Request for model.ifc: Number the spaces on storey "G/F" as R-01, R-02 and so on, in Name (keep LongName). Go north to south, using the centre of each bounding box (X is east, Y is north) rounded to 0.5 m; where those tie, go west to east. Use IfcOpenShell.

First a look at what the model holds.

```python
import ifcopenshell
import ifcopenshell.util.element
import ifcopenshell.util.placement

model = ifcopenshell.open("model.ifc")
print(model.schema)
storey = next(s for s in model.by_type("IfcBuildingStorey") if s.Name == "G/F")
spaces = [e for e in ifcopenshell.util.element.get_decomposition(storey) if e.is_a("IfcSpace")]
for e in sorted(spaces, key=lambda e: e.id()):
    origin = ifcopenshell.util.placement.get_local_placement(e.ObjectPlacement)[:3, 3]
    print(e.id(), e.Name, e.LongName, origin.round(2) + 0.0, sep=" | ")
```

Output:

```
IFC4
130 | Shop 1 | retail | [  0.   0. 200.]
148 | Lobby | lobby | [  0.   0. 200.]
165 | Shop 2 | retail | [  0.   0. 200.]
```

```python
import ifcopenshell
import ifcopenshell.geom
import ifcopenshell.util.element
import ifcopenshell.util.shape

model = ifcopenshell.open("model.ifc")
settings = ifcopenshell.geom.settings()
settings.set("use-world-coords", True)


def centre(element):
    shape = ifcopenshell.geom.create_shape(settings, element)
    return ifcopenshell.util.shape.get_bbox_centroid(shape.geometry)


storey = next(s for s in model.by_type("IfcBuildingStorey") if s.Name == "G/F")
spaces = [e for e in ifcopenshell.util.element.get_decomposition(storey) if e.is_a("IfcSpace")]

# Insertion points can sit at a corner or the storey origin, so sort by the geometry (in metres).
centres = {e: centre(e) for e in spaces}
spaces.sort(key=lambda e: (-round(centres[e][1] / 0.5), centres[e][0]))

for i, e in enumerate(spaces, start=1):
    number = f"R-{i:02d}"
    e.Name = number
    print(e.id(), number)

model.write("model_v2.ifc")
```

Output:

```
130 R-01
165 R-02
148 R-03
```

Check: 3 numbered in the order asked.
